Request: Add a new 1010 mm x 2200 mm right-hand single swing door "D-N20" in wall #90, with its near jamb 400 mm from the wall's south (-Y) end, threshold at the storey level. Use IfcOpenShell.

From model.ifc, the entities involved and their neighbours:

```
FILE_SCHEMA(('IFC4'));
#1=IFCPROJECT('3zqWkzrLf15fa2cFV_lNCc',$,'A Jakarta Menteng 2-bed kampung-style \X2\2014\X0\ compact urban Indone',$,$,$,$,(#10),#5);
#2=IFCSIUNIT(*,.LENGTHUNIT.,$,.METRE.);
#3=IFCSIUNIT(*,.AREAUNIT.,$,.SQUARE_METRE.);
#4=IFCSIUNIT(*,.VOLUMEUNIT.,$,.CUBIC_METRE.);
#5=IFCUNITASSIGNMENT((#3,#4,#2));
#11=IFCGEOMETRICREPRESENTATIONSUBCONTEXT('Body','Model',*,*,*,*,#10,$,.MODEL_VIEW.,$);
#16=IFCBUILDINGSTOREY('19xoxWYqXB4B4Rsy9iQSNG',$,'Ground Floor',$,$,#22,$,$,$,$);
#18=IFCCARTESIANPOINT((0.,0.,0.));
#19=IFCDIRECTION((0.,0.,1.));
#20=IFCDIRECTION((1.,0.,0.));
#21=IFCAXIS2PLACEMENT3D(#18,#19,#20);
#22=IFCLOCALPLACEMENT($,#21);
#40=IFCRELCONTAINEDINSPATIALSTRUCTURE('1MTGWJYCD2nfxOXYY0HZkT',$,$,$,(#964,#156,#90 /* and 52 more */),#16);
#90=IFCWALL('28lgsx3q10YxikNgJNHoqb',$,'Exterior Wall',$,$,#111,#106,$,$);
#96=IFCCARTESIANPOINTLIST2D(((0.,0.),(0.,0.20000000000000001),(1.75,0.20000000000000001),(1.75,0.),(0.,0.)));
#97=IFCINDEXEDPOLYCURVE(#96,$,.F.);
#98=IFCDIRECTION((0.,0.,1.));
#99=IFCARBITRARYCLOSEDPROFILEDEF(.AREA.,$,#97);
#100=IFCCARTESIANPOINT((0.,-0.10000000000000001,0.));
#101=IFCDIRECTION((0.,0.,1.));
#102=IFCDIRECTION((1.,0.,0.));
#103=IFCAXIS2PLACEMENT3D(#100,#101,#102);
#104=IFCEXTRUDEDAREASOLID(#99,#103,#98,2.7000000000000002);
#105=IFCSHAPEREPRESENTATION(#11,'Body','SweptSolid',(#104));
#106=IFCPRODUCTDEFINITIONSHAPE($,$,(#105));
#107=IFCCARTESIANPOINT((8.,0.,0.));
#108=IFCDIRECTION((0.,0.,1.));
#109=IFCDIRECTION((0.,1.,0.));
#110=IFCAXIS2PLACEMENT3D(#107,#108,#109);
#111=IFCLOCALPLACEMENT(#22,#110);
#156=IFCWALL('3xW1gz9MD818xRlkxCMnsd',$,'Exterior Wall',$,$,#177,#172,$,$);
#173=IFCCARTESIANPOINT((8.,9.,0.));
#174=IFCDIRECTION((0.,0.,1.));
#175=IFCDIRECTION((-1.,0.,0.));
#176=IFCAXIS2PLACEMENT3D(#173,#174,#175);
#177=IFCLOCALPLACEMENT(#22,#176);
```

```python
import numpy as np
import ifcopenshell
import ifcopenshell.api.feature
import ifcopenshell.api.geometry
import ifcopenshell.api.root
import ifcopenshell.api.spatial
import ifcopenshell.geom
import ifcopenshell.util.element
import ifcopenshell.util.placement
import ifcopenshell.util.representation
import ifcopenshell.util.shape
import ifcopenshell.util.unit

model = ifcopenshell.open("model.ifc")
unit_scale = ifcopenshell.util.unit.calculate_unit_scale(model)
settings = ifcopenshell.geom.settings()


def volume(element):
    """Net volume in cubic metres, openings subtracted."""
    shape = ifcopenshell.geom.create_shape(settings, element)
    return ifcopenshell.util.shape.get_volume(shape.geometry)


wall = model.by_guid("28lgsx3q10YxikNgJNHoqb")
storey = ifcopenshell.util.element.get_container(wall, ifc_class="IfcBuildingStorey")
context = ifcopenshell.util.representation.get_context(model, "Model", "Body", "MODEL_VIEW")
before = volume(wall)

width, height, from_end, sill = 1.01, 2.2, 0.4, 0.0  # metres

# The wall runs along its own X axis, and the end named is its -X end.
wall_shape = ifcopenshell.geom.create_shape(settings, wall)
x, y, z = ifcopenshell.util.shape.get_vertices(wall_shape.geometry).T
start = x.min() + from_end
face, thickness = float(y.min()), float(y.max() - y.min())
wall_matrix = ifcopenshell.util.placement.get_local_placement(wall.ObjectPlacement)
level = ifcopenshell.util.placement.get_local_placement(storey.ObjectPlacement)[2, 3]


def in_wall(x, y):
    """Placement at x, y metres in the wall's axes, at sill height."""
    matrix = wall_matrix.copy()
    matrix[:, 3] = wall_matrix @ np.array([x / unit_scale, y / unit_scale, 0.0, 1.0])
    matrix[2, 3] = level + sill / unit_scale
    return matrix


# Opening: a box that overshoots both wall faces by 50 mm.
opening = ifcopenshell.api.root.create_entity(model, ifc_class="IfcOpeningElement", predefined_type="OPENING")
box = ifcopenshell.api.geometry.add_wall_representation(
    model, context=context, length=width, height=height, thickness=thickness + 0.1
)
ifcopenshell.api.geometry.assign_representation(model, product=opening, representation=box)
ifcopenshell.api.geometry.edit_object_placement(model, product=opening, matrix=in_wall(start, face - 0.05), is_si=False)
ifcopenshell.api.feature.add_feature(model, feature=opening, element=wall)

door = ifcopenshell.api.root.create_entity(model, ifc_class="IfcDoor", name="D-N20", predefined_type="DOOR")
door.OverallWidth, door.OverallHeight = width / unit_scale, height / unit_scale
door.OperationType = "SINGLE_SWING_RIGHT"
body = ifcopenshell.api.geometry.add_door_representation(
    model,
    context=context,
    overall_width=door.OverallWidth,
    overall_height=door.OverallHeight,
    operation_type="SINGLE_SWING_RIGHT",
    lining_properties={"LiningDepth": thickness / unit_scale, "ThresholdDepth": thickness / unit_scale},
)
ifcopenshell.api.geometry.assign_representation(model, product=door, representation=body)
ifcopenshell.api.spatial.assign_container(model, products=[door], relating_structure=storey)
ifcopenshell.api.feature.add_filling(model, opening=opening, element=door)

# The lining spans the wall, so the door starts at the wall face.
ifcopenshell.api.geometry.edit_object_placement(model, product=door, matrix=in_wall(start, face), is_si=False)

after = volume(wall)

print(f"wall volume {before:.3f} -> {after:.3f} m3")

model.write("model_rev.ifc")
```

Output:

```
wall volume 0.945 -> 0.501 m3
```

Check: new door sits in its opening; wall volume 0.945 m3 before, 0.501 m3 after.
